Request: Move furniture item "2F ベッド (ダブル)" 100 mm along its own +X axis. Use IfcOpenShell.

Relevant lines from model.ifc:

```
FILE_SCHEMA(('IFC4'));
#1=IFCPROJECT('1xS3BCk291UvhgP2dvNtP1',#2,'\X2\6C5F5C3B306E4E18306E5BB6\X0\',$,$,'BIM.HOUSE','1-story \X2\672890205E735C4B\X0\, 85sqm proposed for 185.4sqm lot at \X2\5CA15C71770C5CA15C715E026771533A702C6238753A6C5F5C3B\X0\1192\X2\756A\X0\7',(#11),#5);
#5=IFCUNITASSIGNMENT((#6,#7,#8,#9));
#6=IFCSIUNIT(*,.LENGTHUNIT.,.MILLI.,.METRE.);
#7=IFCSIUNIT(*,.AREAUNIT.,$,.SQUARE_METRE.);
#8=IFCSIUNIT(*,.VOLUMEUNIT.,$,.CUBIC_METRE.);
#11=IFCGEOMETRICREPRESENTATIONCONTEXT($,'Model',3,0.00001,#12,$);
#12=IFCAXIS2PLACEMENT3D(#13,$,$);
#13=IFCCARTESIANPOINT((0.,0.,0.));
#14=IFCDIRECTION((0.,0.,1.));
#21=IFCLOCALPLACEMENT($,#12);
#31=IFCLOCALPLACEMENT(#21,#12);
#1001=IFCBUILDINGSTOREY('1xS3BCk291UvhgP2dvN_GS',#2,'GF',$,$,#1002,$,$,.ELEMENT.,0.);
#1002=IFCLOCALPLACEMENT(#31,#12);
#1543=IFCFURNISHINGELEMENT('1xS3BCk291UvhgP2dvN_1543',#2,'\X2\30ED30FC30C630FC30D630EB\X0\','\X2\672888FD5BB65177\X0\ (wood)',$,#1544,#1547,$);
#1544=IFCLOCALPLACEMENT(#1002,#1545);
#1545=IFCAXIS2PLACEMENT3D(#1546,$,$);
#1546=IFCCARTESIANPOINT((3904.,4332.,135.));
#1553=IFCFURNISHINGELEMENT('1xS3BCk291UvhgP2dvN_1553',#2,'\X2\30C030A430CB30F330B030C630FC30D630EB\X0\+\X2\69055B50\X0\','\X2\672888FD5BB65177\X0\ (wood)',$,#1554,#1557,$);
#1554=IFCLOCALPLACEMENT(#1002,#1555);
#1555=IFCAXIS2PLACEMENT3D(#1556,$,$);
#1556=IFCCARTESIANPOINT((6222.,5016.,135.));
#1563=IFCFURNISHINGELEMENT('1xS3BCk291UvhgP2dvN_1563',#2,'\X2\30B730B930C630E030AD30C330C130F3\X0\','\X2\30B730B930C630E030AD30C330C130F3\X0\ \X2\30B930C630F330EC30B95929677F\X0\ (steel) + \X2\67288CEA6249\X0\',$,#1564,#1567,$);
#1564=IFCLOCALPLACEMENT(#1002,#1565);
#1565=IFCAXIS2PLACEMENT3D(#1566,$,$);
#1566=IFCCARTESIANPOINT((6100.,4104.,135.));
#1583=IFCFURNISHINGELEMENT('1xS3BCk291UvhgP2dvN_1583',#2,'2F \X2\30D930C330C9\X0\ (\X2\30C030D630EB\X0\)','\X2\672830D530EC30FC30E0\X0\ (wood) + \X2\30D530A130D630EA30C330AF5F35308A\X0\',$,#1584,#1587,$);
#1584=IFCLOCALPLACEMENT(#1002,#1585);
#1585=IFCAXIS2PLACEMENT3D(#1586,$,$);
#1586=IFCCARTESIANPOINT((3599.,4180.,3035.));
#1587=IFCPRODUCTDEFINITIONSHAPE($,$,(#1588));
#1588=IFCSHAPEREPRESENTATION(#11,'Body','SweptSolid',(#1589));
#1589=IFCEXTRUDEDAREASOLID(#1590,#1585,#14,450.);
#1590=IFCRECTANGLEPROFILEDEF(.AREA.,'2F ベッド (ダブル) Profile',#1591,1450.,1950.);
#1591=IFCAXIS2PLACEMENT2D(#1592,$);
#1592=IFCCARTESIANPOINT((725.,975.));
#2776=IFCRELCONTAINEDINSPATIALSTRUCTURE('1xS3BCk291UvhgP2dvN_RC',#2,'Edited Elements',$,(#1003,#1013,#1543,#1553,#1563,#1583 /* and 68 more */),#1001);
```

```python
import ifcopenshell
import ifcopenshell.api.geometry
import ifcopenshell.util.placement

model = ifcopenshell.open("model.ifc")

item = model.by_guid("1xS3BCk291UvhgP2dvN_1583")
matrix = ifcopenshell.util.placement.get_local_placement(item.ObjectPlacement)
matrix[:3, 3] += matrix[:3, 0] * 100.0
ifcopenshell.api.geometry.edit_object_placement(model, product=item, matrix=matrix, is_si=False)

print(ifcopenshell.util.placement.get_local_placement(item.ObjectPlacement).round(3) + 0.0)

model.write("model_edited.ifc")
```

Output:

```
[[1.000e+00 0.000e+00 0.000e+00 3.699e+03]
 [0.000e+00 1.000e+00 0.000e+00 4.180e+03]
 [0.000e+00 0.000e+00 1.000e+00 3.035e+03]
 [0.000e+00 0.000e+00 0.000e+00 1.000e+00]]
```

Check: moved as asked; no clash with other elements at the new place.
